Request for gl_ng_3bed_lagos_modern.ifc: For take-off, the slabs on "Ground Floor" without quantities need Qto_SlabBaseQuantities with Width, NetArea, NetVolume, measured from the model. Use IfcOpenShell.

First a look at what the model holds.

```python
import ifcopenshell
import ifcopenshell.util.element
import ifcopenshell.util.unit

model = ifcopenshell.open("gl_ng_3bed_lagos_modern.ifc")
print(model.schema)
for unit_type in ("LENGTHUNIT", "AREAUNIT", "VOLUMEUNIT"):
    print(unit_type, ifcopenshell.util.unit.calculate_unit_scale(model, unit_type))
storey = next(s for s in model.by_type("IfcBuildingStorey") if s.Name == "Ground Floor")
slabs = [e for e in ifcopenshell.util.element.get_decomposition(storey) if e.is_a("IfcSlab")]
for e in sorted(slabs, key=lambda e: e.id()):
    print(e.id(), e.is_a(), e.Name, list(ifcopenshell.util.element.get_psets(e, qtos_only=True)), sep=" | ")
```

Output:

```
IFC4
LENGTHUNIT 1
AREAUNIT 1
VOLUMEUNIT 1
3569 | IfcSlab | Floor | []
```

```python
import ifcopenshell
import ifcopenshell.api.pset
import ifcopenshell.geom
import ifcopenshell.util.element
import ifcopenshell.util.shape
import ifcopenshell.util.unit

model = ifcopenshell.open("gl_ng_3bed_lagos_modern.ifc")
unit_scale = ifcopenshell.util.unit.calculate_unit_scale(model)
area_scale = ifcopenshell.util.unit.calculate_unit_scale(model, "AREAUNIT")
volume_scale = ifcopenshell.util.unit.calculate_unit_scale(model, "VOLUMEUNIT")
settings = ifcopenshell.geom.settings()

storey = next(s for s in model.by_type("IfcBuildingStorey") if s.Name == "Ground Floor")
slabs = [e for e in ifcopenshell.util.element.get_decomposition(storey) if e.is_a("IfcSlab")]

for e in sorted(slabs, key=lambda e: e.id()):
    if ifcopenshell.util.element.get_psets(e, qtos_only=True, should_inherit=False):
        continue
    # Geometry comes back in metres, in the element's own axes.
    shape = ifcopenshell.geom.create_shape(settings, e)
    values = {
        "Width": ifcopenshell.util.shape.get_z(shape.geometry) / unit_scale,
        "NetArea": ifcopenshell.util.shape.get_footprint_area(shape.geometry) / area_scale,
        "NetVolume": ifcopenshell.util.shape.get_volume(shape.geometry) / volume_scale,
    }
    qto = ifcopenshell.api.pset.add_qto(model, product=e, name="Qto_SlabBaseQuantities")
    ifcopenshell.api.pset.edit_qto(model, qto=qto, properties=values)
    print(e.id(), {k: round(v, 3) for k, v in values.items()})

model.write("gl_ng_3bed_lagos_modern_updated.ifc")
```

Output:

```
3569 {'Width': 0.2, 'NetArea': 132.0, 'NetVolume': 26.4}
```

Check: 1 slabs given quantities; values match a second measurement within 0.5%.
